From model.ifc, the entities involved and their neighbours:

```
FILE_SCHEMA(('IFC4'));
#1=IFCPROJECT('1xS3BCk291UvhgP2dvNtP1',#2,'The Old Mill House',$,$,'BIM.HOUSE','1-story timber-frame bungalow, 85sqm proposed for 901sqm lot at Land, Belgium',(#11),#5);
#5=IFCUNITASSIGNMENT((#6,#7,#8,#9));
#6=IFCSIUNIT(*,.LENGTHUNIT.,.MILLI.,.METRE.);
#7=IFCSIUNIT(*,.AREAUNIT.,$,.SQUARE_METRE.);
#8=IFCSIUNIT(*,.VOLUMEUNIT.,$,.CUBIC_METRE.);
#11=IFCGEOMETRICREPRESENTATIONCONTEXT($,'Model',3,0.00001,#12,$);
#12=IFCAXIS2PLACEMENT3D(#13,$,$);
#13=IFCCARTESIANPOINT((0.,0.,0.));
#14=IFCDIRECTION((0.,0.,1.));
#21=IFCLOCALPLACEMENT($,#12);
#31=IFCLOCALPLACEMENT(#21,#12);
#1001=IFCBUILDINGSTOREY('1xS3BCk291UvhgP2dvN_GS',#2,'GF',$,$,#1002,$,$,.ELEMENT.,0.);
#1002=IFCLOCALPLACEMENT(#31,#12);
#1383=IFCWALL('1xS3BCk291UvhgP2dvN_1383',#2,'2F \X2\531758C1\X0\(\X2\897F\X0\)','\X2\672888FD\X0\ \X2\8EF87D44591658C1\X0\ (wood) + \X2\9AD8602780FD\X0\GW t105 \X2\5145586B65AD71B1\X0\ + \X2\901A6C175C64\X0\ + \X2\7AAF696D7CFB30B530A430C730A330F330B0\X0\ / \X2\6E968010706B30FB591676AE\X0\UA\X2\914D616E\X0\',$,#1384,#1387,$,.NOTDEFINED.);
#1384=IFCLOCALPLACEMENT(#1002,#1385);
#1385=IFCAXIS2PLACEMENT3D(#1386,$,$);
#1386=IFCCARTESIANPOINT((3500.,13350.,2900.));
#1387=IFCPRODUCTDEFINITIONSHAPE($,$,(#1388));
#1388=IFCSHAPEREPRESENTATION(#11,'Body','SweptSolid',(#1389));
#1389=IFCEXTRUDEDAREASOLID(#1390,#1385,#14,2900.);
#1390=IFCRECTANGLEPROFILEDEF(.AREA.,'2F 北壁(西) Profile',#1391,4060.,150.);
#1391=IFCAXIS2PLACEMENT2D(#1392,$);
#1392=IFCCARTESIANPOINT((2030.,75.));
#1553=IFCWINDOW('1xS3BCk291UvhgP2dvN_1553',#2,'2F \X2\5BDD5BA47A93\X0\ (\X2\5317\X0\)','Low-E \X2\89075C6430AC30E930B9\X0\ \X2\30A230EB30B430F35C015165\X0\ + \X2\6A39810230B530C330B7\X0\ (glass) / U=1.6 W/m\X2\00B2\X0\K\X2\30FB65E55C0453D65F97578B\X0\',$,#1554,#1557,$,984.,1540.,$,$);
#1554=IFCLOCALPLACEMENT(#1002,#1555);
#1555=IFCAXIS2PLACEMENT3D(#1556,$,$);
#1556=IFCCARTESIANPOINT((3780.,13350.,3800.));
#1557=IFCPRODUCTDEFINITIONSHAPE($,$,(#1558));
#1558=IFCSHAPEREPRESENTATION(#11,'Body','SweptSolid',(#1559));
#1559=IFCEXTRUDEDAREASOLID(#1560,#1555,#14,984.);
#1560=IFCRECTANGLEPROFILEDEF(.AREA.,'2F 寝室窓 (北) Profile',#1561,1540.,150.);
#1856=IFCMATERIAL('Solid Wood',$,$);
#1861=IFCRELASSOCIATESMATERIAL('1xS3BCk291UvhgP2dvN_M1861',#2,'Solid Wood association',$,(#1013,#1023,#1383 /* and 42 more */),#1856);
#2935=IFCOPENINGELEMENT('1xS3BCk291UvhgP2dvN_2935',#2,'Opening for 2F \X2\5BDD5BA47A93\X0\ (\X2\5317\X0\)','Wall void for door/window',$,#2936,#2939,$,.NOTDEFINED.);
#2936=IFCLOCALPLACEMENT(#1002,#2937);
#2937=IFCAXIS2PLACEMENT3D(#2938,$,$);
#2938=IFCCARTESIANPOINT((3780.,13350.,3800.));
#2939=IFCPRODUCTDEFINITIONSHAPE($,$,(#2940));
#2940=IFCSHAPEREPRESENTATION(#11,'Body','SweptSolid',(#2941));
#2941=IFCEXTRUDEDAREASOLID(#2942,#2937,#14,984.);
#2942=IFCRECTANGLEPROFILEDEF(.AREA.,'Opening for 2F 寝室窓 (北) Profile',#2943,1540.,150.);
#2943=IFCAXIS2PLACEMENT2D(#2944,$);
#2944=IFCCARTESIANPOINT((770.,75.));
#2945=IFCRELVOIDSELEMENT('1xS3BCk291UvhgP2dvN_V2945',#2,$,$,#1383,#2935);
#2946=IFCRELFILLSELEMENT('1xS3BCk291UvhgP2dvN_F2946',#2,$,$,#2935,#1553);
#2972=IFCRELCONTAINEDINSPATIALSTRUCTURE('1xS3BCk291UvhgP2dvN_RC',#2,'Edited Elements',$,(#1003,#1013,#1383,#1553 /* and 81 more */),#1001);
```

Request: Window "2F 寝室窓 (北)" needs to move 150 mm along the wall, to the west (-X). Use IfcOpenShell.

```python
import ifcopenshell
import ifcopenshell.api.geometry
import ifcopenshell.util.placement

model = ifcopenshell.open("model.ifc")

window = model.by_guid("1xS3BCk291UvhgP2dvN_1553")
opening = window.FillsVoids[0].RelatingOpeningElement
wall = opening.VoidsElements[0].RelatingBuildingElement

wall_matrix = ifcopenshell.util.placement.get_local_placement(wall.ObjectPlacement)
shift = wall_matrix[:3, 0] * -150.0
before = ifcopenshell.util.placement.get_local_placement(window.ObjectPlacement)[:3, 3].copy()

# The window is not placed relative to its opening, so move both.
for product in (opening, window):
    matrix = ifcopenshell.util.placement.get_local_placement(product.ObjectPlacement)
    matrix[:3, 3] += shift
    ifcopenshell.api.geometry.edit_object_placement(model, product=product, matrix=matrix, is_si=False)

after = ifcopenshell.util.placement.get_local_placement(window.ObjectPlacement)[:3, 3]
print("window moved by", (after - before).round(3) + 0.0)

model.write("model-out.ifc")
```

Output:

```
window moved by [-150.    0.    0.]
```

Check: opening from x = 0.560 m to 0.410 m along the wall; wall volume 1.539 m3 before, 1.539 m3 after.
